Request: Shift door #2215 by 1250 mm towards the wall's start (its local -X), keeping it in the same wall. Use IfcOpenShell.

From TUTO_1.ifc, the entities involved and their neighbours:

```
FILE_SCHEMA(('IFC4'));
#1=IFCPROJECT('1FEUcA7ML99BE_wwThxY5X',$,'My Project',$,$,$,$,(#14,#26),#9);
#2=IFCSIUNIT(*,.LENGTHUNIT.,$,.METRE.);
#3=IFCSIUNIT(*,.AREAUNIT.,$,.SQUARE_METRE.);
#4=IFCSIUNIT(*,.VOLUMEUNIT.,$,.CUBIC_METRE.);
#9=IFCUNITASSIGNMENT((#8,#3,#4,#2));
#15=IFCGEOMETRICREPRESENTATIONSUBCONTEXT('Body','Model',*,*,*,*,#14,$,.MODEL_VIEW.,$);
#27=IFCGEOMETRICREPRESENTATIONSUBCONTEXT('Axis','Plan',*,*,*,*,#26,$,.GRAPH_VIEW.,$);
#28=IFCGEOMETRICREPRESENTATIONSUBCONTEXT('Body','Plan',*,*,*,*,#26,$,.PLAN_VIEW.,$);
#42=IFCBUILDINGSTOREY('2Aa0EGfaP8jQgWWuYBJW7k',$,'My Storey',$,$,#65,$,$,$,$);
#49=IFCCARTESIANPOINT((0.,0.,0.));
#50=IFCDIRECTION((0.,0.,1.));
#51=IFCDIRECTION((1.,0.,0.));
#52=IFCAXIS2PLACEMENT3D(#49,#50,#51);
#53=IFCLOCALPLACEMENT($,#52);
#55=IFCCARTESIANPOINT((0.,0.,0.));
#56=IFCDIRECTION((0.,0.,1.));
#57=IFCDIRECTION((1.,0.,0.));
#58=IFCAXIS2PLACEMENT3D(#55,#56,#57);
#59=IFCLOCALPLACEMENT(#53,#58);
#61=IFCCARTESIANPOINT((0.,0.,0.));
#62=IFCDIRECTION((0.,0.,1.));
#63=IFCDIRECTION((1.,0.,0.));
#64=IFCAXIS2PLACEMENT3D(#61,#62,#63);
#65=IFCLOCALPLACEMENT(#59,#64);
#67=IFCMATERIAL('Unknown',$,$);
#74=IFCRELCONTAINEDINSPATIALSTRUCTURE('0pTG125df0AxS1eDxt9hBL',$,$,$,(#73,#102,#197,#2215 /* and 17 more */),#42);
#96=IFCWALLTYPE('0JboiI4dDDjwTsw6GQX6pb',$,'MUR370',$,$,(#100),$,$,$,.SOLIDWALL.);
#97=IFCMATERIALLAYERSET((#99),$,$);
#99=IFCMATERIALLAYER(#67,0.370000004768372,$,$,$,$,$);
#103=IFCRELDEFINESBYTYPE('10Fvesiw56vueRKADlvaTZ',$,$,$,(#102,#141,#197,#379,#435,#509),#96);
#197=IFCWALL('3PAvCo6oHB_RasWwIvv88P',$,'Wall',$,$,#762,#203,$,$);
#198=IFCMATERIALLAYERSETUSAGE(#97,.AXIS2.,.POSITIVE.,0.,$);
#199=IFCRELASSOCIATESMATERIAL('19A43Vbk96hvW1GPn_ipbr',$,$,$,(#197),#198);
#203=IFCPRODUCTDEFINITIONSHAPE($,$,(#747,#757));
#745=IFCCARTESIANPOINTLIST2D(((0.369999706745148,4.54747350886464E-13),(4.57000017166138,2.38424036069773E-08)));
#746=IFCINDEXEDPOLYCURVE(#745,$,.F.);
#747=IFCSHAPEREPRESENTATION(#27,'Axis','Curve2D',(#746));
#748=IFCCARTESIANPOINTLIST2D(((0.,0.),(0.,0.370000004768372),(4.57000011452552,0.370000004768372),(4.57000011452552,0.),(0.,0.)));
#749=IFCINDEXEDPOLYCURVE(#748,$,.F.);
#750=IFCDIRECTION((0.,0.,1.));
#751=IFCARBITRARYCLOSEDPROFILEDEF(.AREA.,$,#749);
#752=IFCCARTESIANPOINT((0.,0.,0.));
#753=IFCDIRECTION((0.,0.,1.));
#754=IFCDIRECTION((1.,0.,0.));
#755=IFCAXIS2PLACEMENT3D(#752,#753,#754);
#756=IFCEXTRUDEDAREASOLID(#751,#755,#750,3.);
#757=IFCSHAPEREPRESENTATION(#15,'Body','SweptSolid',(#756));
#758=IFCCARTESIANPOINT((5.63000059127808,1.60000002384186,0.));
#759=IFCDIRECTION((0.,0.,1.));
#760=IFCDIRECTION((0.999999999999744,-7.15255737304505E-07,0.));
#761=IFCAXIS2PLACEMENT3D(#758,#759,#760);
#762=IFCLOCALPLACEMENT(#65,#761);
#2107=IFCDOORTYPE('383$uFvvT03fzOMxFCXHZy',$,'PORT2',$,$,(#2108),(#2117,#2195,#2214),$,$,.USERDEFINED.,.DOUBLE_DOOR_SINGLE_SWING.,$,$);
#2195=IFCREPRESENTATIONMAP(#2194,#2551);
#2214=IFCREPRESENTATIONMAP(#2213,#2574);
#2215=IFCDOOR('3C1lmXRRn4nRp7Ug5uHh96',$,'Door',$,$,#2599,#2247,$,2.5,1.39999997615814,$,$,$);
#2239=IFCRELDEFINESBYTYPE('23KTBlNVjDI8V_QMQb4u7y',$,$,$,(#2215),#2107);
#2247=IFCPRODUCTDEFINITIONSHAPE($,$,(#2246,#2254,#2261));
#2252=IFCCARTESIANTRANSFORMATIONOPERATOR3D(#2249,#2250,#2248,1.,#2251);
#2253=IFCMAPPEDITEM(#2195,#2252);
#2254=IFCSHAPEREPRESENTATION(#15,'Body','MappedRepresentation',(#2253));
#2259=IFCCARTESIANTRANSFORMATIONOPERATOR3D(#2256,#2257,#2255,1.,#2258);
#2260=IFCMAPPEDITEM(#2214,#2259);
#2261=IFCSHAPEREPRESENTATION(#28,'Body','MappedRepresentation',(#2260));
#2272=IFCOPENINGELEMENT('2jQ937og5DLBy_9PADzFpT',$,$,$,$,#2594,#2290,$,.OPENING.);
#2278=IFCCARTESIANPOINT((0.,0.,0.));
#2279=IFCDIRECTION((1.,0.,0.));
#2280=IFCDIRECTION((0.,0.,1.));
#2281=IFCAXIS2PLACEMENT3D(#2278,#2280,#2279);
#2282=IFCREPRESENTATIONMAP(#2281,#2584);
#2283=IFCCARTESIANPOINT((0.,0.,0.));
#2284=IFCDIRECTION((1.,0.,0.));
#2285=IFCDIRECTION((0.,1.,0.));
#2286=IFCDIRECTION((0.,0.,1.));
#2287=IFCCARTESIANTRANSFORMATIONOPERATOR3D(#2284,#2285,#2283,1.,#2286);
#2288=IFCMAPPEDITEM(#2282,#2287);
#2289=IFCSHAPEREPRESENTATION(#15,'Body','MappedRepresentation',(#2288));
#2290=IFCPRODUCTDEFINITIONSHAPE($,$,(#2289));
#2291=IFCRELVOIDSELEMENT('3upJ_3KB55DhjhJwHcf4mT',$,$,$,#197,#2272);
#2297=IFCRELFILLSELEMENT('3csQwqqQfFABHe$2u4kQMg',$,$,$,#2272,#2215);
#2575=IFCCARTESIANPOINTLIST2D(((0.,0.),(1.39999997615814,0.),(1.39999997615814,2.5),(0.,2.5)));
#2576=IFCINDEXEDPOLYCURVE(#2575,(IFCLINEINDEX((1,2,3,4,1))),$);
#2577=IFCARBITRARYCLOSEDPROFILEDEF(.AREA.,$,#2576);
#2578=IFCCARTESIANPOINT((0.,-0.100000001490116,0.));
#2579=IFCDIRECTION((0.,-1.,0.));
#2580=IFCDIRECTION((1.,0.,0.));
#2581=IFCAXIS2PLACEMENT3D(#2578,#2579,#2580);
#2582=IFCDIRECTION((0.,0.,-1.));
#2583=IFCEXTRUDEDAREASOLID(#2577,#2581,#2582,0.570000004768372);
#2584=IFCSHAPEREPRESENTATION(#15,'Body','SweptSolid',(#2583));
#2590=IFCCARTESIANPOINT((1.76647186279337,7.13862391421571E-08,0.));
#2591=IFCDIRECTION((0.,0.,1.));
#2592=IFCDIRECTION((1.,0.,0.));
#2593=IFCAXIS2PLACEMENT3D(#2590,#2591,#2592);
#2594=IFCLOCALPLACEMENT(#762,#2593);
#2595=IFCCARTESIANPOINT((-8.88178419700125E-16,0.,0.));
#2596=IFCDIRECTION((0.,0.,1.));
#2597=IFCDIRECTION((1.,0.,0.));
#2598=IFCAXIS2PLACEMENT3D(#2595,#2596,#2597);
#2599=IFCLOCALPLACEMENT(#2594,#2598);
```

```python
import ifcopenshell
import ifcopenshell.api.geometry
import ifcopenshell.util.placement
import ifcopenshell.util.unit

model = ifcopenshell.open("TUTO_1.ifc")
unit_scale = ifcopenshell.util.unit.calculate_unit_scale(model)

door = model.by_guid("3C1lmXRRn4nRp7Ug5uHh96")
opening = door.FillsVoids[0].RelatingOpeningElement
wall = opening.VoidsElements[0].RelatingBuildingElement

wall_matrix = ifcopenshell.util.placement.get_local_placement(wall.ObjectPlacement)
shift = wall_matrix[:3, 0] * -1.25 / unit_scale
before = ifcopenshell.util.placement.get_local_placement(door.ObjectPlacement)[:3, 3].copy()

# The door is placed relative to its opening, so it follows when the opening moves.
matrix = ifcopenshell.util.placement.get_local_placement(opening.ObjectPlacement)
matrix[:3, 3] += shift
ifcopenshell.api.geometry.edit_object_placement(
    model, product=opening, matrix=matrix, is_si=False, should_transform_children=True
)

after = ifcopenshell.util.placement.get_local_placement(door.ObjectPlacement)[:3, 3]
print("door moved by", (after - before).round(3) + 0.0)

model.write("TUTO_1_v2.ifc")
```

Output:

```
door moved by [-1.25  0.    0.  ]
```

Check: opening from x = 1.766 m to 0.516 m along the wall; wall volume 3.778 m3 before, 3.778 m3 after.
